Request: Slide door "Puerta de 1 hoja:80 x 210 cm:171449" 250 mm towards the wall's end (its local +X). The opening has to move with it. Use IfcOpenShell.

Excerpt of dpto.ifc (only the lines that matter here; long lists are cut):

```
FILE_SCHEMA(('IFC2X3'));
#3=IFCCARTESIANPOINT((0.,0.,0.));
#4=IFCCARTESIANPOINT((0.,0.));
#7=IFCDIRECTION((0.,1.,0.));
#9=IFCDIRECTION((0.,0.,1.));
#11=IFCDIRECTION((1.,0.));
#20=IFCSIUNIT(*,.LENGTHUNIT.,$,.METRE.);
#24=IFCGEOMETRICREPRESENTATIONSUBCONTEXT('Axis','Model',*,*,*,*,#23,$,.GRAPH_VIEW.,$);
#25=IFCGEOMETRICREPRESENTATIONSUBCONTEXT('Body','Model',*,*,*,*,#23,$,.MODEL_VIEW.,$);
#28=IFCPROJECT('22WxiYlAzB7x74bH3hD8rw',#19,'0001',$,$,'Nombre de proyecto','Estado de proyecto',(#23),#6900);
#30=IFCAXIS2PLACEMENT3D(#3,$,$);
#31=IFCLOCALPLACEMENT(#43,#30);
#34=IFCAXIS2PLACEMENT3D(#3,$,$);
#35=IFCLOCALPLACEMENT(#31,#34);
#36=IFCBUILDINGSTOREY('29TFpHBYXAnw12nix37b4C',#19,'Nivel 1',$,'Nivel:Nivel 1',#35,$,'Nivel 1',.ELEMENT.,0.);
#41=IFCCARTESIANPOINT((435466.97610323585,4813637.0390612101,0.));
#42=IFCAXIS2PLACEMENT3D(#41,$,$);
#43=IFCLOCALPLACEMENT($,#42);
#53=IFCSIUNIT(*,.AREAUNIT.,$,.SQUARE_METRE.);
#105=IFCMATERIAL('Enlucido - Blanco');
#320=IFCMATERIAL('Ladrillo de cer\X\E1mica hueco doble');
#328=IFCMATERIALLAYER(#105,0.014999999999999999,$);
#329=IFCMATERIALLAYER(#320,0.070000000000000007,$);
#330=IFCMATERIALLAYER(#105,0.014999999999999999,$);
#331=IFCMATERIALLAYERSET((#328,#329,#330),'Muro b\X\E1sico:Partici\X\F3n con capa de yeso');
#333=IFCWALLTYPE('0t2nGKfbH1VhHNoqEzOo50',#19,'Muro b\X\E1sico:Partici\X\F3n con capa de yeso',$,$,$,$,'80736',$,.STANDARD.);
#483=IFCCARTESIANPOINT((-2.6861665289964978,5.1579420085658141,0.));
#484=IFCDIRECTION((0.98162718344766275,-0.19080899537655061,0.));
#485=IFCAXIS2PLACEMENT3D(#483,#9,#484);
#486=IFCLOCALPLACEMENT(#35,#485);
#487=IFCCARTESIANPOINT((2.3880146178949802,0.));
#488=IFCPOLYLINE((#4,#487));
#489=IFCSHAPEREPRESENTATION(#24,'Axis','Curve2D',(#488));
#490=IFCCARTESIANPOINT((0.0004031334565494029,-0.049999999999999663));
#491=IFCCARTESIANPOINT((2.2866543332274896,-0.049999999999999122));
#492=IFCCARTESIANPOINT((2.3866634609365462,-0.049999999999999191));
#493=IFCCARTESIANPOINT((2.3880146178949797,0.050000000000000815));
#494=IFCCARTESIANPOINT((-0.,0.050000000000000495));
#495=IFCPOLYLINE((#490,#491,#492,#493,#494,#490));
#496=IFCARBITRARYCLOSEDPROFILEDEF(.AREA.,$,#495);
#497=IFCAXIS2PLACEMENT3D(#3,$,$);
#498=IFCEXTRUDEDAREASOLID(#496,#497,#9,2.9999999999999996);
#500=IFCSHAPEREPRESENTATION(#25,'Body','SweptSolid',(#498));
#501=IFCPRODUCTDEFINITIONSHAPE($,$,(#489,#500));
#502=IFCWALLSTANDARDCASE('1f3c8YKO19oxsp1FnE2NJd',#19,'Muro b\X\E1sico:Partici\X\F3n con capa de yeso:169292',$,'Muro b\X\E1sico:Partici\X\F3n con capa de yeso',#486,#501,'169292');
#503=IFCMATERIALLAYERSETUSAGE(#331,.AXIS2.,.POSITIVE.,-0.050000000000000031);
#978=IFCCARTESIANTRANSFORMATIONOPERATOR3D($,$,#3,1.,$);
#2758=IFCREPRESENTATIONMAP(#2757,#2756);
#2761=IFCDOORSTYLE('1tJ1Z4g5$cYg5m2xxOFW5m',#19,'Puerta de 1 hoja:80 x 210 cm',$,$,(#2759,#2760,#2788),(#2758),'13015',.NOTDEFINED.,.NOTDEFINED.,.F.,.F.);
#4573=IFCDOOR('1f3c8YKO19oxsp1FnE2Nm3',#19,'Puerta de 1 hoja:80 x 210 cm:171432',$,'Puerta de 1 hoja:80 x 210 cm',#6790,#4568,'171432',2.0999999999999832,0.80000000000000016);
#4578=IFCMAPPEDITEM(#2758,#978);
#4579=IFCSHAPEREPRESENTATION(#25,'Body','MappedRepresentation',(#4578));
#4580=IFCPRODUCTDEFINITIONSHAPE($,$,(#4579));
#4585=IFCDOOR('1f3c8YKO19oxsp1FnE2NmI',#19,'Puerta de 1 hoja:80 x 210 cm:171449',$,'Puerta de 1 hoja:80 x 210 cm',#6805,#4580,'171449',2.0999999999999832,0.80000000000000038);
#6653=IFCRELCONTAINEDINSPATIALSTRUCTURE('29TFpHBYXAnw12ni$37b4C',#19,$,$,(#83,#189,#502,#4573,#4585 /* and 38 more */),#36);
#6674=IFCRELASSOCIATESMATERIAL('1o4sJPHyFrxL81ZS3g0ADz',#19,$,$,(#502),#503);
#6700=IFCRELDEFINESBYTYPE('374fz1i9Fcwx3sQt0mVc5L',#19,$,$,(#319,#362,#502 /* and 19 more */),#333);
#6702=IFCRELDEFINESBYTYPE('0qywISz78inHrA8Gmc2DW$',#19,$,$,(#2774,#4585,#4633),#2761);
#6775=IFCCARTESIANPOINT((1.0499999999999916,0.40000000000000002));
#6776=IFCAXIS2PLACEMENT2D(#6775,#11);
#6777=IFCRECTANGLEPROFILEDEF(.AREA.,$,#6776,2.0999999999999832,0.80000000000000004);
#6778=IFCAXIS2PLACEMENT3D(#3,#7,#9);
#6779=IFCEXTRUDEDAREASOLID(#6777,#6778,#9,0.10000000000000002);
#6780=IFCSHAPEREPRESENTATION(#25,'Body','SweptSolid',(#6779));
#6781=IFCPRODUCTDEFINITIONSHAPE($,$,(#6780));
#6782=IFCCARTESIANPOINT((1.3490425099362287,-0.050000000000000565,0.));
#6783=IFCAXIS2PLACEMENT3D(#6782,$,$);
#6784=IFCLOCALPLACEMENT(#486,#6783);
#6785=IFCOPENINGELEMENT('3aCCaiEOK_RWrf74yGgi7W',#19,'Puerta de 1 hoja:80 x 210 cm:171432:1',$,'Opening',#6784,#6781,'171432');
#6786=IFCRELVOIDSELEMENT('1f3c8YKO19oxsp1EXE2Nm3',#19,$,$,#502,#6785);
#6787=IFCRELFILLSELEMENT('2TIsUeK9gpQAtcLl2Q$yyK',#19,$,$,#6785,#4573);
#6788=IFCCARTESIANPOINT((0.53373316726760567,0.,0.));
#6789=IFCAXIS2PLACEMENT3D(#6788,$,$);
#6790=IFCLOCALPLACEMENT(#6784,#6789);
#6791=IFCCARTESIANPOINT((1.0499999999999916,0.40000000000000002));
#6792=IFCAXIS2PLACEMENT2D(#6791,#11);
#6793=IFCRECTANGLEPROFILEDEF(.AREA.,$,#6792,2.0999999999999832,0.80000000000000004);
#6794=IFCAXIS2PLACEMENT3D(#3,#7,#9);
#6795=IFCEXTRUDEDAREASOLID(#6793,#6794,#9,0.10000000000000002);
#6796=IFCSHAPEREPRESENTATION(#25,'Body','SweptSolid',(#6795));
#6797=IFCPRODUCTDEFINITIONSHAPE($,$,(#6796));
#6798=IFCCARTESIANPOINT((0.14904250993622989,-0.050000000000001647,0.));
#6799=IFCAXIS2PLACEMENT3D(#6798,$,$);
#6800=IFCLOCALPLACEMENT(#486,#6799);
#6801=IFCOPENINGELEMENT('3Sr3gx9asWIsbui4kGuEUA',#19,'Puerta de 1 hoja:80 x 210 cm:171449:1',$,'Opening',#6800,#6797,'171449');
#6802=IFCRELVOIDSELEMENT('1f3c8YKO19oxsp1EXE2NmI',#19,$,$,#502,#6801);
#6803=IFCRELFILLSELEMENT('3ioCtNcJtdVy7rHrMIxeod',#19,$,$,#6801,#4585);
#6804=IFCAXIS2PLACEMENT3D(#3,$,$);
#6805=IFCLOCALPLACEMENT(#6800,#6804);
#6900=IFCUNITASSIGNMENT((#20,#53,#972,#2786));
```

```python
import ifcopenshell
import ifcopenshell.api.geometry
import ifcopenshell.util.placement
import ifcopenshell.util.unit

model = ifcopenshell.open("dpto.ifc")
unit_scale = ifcopenshell.util.unit.calculate_unit_scale(model)

door = model.by_guid("1f3c8YKO19oxsp1FnE2NmI")
opening = door.FillsVoids[0].RelatingOpeningElement
wall = opening.VoidsElements[0].RelatingBuildingElement

wall_matrix = ifcopenshell.util.placement.get_local_placement(wall.ObjectPlacement)
shift = wall_matrix[:3, 0] * 0.25 / unit_scale
before = ifcopenshell.util.placement.get_local_placement(door.ObjectPlacement)[:3, 3].copy()

# The door is placed relative to its opening, so it follows when the opening moves.
matrix = ifcopenshell.util.placement.get_local_placement(opening.ObjectPlacement)
matrix[:3, 3] += shift
ifcopenshell.api.geometry.edit_object_placement(
    model, product=opening, matrix=matrix, is_si=False, should_transform_children=True
)

after = ifcopenshell.util.placement.get_local_placement(door.ObjectPlacement)[:3, 3]
print("door moved by", (after - before).round(3) + 0.0)

model.write("dpto_rev.ifc")
```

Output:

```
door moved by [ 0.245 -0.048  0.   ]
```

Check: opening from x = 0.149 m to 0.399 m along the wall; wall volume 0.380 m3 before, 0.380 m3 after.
